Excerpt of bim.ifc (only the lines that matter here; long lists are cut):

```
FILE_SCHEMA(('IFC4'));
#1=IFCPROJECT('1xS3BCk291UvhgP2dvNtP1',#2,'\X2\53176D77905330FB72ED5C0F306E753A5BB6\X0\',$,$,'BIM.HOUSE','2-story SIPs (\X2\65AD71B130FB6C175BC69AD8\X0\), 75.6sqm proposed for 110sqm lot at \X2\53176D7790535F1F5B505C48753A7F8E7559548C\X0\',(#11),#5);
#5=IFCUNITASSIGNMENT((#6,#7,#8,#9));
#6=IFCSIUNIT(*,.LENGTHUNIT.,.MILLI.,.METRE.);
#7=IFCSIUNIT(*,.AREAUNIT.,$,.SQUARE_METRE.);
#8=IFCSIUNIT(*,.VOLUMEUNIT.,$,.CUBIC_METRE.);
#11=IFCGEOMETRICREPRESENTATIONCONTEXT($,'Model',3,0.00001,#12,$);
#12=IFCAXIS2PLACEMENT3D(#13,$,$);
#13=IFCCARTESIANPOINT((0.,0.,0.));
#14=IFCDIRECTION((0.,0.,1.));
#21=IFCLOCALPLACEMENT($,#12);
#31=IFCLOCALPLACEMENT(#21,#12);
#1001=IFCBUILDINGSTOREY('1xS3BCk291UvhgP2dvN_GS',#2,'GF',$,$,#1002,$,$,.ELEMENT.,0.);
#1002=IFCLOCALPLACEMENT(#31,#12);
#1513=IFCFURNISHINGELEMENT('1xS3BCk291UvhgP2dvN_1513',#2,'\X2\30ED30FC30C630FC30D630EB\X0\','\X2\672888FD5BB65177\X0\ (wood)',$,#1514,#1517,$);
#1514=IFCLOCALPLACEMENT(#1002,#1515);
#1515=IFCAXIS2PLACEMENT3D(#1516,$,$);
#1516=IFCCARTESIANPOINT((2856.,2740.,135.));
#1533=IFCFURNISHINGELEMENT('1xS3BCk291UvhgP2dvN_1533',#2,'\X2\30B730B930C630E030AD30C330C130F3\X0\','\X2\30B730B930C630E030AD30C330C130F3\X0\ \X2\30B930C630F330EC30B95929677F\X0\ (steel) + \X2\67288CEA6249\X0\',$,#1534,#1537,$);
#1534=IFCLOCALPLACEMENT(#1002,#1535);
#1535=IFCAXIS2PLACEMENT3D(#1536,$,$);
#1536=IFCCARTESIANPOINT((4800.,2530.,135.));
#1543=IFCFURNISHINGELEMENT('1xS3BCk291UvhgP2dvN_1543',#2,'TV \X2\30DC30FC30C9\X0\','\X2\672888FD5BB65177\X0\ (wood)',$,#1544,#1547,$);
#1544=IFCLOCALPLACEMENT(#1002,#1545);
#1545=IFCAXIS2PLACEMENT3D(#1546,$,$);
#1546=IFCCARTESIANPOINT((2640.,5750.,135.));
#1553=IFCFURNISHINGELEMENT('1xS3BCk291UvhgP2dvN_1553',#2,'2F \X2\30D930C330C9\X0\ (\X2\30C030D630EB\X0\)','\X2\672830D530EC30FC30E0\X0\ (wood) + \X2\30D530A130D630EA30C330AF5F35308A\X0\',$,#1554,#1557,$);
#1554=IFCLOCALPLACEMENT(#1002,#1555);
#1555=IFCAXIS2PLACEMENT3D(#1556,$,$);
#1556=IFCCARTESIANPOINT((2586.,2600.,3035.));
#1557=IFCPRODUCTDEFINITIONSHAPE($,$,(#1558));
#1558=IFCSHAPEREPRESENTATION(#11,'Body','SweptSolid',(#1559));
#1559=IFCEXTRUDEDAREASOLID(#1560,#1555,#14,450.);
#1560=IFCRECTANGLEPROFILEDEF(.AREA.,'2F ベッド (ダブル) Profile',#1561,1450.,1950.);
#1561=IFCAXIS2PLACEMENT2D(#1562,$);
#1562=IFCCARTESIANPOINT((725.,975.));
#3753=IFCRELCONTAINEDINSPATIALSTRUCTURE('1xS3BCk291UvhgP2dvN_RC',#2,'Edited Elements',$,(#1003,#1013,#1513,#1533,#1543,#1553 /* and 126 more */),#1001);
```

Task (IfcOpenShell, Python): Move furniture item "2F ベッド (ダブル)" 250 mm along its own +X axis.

```python
import ifcopenshell
import ifcopenshell.api.geometry
import ifcopenshell.util.placement
import ifcopenshell.util.unit

model = ifcopenshell.open("bim.ifc")
unit_scale = ifcopenshell.util.unit.calculate_unit_scale(model)

item = model.by_guid("1xS3BCk291UvhgP2dvN_1553")
matrix = ifcopenshell.util.placement.get_local_placement(item.ObjectPlacement)
matrix[:3, 3] += matrix[:3, 0] * 0.25 / unit_scale
ifcopenshell.api.geometry.edit_object_placement(model, product=item, matrix=matrix, is_si=False)

print(ifcopenshell.util.placement.get_local_placement(item.ObjectPlacement).round(3) + 0.0)

model.write("bim-out.ifc")
```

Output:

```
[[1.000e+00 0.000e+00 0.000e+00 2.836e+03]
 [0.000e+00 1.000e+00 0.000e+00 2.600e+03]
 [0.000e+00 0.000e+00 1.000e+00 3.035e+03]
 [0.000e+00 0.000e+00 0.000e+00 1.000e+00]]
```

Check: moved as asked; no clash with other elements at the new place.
